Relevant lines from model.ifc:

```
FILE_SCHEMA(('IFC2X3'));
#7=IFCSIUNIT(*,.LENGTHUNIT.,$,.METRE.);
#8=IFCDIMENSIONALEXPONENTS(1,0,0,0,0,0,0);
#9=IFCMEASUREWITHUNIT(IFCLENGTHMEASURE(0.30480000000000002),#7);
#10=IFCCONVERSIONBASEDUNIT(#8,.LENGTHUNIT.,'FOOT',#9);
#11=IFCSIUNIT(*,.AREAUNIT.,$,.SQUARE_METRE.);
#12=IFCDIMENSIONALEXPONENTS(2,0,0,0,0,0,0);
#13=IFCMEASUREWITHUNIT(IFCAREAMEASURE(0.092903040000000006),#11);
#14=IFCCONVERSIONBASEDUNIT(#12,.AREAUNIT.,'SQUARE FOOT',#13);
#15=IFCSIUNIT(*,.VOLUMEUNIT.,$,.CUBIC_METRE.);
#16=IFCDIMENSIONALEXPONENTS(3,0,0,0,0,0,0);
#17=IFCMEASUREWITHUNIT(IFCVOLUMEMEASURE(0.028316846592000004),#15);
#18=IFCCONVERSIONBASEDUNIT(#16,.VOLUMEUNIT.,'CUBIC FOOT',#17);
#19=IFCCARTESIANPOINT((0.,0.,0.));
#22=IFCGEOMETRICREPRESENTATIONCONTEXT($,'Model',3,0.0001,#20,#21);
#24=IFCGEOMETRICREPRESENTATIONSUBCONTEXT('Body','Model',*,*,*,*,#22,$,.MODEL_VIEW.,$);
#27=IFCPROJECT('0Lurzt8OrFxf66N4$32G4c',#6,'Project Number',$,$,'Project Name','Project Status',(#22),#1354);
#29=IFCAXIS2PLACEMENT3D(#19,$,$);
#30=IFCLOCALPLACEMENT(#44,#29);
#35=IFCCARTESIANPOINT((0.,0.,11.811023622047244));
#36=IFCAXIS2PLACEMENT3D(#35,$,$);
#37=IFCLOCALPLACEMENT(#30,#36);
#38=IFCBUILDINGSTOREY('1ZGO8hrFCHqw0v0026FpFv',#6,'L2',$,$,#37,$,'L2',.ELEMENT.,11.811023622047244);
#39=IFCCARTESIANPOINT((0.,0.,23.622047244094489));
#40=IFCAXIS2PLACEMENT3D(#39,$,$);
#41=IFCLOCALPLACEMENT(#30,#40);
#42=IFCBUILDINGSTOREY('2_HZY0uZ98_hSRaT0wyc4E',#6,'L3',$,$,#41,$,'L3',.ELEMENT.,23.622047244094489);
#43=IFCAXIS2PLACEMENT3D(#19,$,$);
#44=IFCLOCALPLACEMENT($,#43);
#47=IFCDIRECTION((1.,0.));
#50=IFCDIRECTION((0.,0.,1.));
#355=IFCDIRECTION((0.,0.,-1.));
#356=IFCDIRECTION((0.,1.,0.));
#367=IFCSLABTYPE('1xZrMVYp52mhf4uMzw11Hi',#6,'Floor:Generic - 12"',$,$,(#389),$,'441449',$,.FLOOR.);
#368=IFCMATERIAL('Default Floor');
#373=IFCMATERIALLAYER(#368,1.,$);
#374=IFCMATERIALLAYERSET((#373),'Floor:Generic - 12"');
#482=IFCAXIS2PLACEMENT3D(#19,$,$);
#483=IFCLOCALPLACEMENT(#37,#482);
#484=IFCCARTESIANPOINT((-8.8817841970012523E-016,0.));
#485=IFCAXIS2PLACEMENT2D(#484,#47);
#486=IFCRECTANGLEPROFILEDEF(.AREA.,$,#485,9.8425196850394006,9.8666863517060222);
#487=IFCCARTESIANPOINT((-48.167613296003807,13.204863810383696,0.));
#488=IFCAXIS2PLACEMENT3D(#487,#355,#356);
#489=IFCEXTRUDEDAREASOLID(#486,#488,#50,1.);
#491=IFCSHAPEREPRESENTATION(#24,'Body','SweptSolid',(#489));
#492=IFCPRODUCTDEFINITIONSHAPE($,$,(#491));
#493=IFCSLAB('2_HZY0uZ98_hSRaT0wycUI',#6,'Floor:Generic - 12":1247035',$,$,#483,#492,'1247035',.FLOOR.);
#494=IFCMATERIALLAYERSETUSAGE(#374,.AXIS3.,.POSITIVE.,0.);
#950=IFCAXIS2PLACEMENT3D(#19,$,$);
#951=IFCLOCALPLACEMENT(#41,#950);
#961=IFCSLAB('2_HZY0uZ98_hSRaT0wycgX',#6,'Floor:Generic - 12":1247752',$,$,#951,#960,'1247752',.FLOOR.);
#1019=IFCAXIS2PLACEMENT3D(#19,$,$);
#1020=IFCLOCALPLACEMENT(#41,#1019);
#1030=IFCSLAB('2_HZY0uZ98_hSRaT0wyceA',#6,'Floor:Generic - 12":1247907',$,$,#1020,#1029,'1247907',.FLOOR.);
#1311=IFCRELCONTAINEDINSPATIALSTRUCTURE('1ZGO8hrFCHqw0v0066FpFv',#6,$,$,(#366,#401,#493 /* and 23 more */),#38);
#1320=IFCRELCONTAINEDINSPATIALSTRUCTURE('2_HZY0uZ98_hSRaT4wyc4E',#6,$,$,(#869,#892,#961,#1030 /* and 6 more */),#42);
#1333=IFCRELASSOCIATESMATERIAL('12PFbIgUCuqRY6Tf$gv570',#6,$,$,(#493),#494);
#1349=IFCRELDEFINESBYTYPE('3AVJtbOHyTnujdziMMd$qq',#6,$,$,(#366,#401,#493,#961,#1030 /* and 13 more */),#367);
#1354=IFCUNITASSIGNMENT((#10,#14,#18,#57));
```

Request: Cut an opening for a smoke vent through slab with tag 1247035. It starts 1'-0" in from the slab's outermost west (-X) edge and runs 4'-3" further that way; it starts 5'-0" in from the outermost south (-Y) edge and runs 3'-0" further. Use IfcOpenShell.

```python
import numpy as np
import ifcopenshell
import ifcopenshell.api.feature
import ifcopenshell.api.geometry
import ifcopenshell.api.root
import ifcopenshell.geom
import ifcopenshell.util.placement
import ifcopenshell.util.representation
import ifcopenshell.util.shape
import ifcopenshell.util.unit

model = ifcopenshell.open("model.ifc")
unit_scale = ifcopenshell.util.unit.calculate_unit_scale(model)
settings = ifcopenshell.geom.settings()


def volume(element):
    """Net volume in cubic metres, openings subtracted."""
    shape = ifcopenshell.geom.create_shape(settings, element)
    return ifcopenshell.util.shape.get_volume(shape.geometry)


slab = model.by_id(493)
before = volume(slab)

# Extent in the slab's own axes, in metres. The edges named are its -X and -Y sides.
slab_shape = ifcopenshell.geom.create_shape(settings, slab)
vertices = ifcopenshell.util.shape.get_vertices(slab_shape.geometry)
x_min, y_min, bottom = vertices.min(axis=0)
top = vertices[:, 2].max()

opening = ifcopenshell.api.root.create_entity(model, ifc_class="IfcOpeningElement", name="Smoke vent opening")
context = ifcopenshell.util.representation.get_context(model, "Model", "Body", "MODEL_VIEW")
width, depth = 1.2954, 0.9144
outline = [(0.0, 0.0), (width, 0.0), (width, depth), (0.0, depth), (0.0, 0.0)]
# Overshoot both faces by 50 mm so the cut is clean.
shape = ifcopenshell.api.geometry.add_slab_representation(
    model, context=context, depth=top - bottom + 0.1, polyline=outline
)
ifcopenshell.api.geometry.assign_representation(model, product=opening, representation=shape)

matrix = ifcopenshell.util.placement.get_local_placement(slab.ObjectPlacement)
matrix[:, 3] = matrix @ np.append(np.array([x_min + 0.3048, y_min + 1.524, bottom - 0.05]) / unit_scale, 1.0)
ifcopenshell.api.geometry.edit_object_placement(model, product=opening, matrix=matrix, is_si=False)
ifcopenshell.api.feature.add_feature(model, feature=opening, element=slab)

after = volume(slab)

print(f"slab volume {before:.3f} -> {after:.3f} m3")

model.write("model_v2.ifc")
```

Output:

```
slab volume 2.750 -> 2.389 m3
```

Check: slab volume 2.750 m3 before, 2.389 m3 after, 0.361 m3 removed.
